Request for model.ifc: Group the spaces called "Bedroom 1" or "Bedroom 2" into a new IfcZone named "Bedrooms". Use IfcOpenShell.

First a look at what the model holds.

```python
import ifcopenshell

model = ifcopenshell.open("model.ifc")
print(model.schema)
seen = {}
for space in model.by_type("IfcSpace"):
    seen[space.LongName] = seen.get(space.LongName, 0) + 1
for name, count in sorted(seen.items(), key=str):
    print(count, "x", name)
print("zones:", [z.Name for z in model.by_type("IfcZone")][:20])
```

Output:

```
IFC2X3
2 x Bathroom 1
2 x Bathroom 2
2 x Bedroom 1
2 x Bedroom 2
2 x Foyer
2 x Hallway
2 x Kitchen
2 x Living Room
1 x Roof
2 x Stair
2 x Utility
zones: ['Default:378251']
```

```python
import ifcopenshell
import ifcopenshell.api.group
import ifcopenshell.api.root

model = ifcopenshell.open("model.ifc")

names = {"Bedroom 1", "Bedroom 2"}
spaces = [s for s in model.by_type("IfcSpace") if s.LongName in names]

zone = ifcopenshell.api.root.create_entity(model, ifc_class="IfcZone", name="Bedrooms")
ifcopenshell.api.group.assign_group(model, products=spaces, group=zone)
print(len(spaces), "spaces in", zone.Name)

model.write("model_edited.ifc")
```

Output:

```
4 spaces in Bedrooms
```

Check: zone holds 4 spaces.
